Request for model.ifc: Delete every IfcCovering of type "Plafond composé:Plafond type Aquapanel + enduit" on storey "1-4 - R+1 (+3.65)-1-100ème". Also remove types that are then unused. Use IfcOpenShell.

First a look at what the model holds.

```python
import ifcopenshell
import ifcopenshell.util.element

model = ifcopenshell.open("model.ifc")
print(model.schema)
storey = next(s for s in model.by_type("IfcBuildingStorey") if s.Name == "1-4 - R+1 (+3.65)-1-100ème")
coverings = [e for e in ifcopenshell.util.element.get_decomposition(storey) if e.is_a("IfcCovering")]
seen = {}
for e in coverings:
    element_type = ifcopenshell.util.element.get_type(e)
    name = element_type.Name if element_type not in (None, e) else None
    seen[name] = seen.get(name, 0) + 1
for name, count in sorted(seen.items(), key=str):
    print(count, "x", name)
```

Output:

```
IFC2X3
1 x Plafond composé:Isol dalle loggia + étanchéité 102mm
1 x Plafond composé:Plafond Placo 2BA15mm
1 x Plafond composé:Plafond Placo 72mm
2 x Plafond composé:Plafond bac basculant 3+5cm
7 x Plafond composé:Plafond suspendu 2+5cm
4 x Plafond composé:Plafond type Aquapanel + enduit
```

```python
import ifcopenshell
import ifcopenshell.api.root
import ifcopenshell.util.element

model = ifcopenshell.open("model.ifc")

storey = next(s for s in model.by_type("IfcBuildingStorey") if s.Name == "1-4 - R+1 (+3.65)-1-100ème")
coverings = [e for e in ifcopenshell.util.element.get_decomposition(storey) if e.is_a("IfcCovering")]
targets = [e for e in coverings if (t := ifcopenshell.util.element.get_type(e)) not in (None, e) and t.Name == "Plafond composé:Plafond type Aquapanel + enduit"]
types = {ifcopenshell.util.element.get_type(e) for e in targets} - {None, *targets}

for e in targets:
    ifcopenshell.api.root.remove_product(model, product=e)
print(len(targets), "removed")

unused = [t for t in types if not ifcopenshell.util.element.get_types(t)]
for t in unused:
    ifcopenshell.api.root.remove_product(model, product=t)
print(len(unused), "unused types removed")

model.write("model_edited.ifc")
```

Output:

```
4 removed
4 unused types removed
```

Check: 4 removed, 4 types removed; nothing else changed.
